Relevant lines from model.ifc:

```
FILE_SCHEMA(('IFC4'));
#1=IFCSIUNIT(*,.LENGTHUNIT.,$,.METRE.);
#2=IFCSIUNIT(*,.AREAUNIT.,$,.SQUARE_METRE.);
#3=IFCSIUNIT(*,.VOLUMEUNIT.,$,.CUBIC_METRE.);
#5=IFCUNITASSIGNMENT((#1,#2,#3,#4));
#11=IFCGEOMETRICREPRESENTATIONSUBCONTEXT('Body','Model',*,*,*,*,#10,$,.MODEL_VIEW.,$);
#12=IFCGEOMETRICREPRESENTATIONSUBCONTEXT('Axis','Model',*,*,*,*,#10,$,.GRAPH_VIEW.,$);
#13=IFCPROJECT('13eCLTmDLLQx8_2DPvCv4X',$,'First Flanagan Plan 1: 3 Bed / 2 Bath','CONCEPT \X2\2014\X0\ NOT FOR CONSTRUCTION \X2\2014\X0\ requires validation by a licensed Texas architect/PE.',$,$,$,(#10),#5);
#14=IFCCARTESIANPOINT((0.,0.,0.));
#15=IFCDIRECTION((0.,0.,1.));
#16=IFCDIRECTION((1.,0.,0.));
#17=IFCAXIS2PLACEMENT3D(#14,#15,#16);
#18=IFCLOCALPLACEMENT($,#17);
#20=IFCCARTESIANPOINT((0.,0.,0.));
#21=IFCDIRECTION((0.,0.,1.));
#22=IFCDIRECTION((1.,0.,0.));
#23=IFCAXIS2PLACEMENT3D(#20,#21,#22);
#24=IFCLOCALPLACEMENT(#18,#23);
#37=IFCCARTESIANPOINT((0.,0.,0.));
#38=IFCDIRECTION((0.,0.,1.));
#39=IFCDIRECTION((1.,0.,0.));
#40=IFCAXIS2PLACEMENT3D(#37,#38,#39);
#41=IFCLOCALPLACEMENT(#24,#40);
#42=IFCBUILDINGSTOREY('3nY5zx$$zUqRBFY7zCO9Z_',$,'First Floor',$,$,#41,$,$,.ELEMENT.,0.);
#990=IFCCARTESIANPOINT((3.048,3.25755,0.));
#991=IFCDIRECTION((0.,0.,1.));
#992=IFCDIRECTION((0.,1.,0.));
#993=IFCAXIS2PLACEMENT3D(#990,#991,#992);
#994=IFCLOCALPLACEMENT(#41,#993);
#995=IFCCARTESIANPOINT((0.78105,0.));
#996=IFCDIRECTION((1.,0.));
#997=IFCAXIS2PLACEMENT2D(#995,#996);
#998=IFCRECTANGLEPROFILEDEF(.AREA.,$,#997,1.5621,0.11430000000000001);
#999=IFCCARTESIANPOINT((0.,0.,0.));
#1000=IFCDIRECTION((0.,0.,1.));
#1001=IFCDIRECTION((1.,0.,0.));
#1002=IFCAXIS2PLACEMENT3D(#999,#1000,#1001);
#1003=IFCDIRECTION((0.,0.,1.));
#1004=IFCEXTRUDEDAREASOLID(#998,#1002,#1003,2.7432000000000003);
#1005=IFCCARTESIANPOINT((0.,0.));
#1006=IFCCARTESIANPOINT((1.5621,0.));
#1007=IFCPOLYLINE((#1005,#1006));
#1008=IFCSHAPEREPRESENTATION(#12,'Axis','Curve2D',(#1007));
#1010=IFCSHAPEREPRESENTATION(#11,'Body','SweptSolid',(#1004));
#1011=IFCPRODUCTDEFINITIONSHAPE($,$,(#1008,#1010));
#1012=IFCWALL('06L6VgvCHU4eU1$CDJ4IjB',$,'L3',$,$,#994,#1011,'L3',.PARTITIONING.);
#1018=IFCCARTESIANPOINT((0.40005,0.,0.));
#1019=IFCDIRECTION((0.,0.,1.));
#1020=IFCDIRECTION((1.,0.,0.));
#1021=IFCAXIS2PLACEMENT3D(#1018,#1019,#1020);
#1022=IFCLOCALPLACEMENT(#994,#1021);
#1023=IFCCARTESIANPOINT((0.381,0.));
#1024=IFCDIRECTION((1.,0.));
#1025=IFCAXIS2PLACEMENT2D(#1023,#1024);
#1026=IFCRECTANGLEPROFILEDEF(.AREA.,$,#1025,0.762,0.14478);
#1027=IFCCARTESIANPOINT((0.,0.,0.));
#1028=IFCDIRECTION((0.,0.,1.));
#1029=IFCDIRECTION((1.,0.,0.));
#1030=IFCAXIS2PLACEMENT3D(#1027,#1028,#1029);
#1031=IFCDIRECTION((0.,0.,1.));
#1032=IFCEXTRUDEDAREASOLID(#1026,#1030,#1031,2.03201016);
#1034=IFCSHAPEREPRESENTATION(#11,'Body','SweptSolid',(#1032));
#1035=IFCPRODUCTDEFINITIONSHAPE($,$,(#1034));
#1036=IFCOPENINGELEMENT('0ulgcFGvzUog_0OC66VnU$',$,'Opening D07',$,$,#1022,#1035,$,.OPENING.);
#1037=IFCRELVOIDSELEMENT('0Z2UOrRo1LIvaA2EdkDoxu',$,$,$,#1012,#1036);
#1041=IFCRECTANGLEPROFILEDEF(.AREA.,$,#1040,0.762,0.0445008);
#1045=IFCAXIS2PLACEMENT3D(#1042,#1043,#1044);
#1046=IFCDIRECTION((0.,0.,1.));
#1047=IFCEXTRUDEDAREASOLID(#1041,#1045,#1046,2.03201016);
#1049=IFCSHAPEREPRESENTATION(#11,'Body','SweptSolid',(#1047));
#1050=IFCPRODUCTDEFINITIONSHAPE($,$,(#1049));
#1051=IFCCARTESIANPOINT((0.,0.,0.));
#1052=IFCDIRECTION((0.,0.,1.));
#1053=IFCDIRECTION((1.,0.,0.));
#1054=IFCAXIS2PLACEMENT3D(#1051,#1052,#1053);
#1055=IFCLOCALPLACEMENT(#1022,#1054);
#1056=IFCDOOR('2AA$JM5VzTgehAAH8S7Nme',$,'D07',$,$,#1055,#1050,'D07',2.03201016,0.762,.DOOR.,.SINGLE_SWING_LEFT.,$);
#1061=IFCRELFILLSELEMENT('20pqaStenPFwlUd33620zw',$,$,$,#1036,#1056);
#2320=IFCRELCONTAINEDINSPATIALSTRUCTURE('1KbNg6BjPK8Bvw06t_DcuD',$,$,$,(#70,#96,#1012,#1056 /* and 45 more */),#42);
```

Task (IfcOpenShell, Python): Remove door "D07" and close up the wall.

```python
import ifcopenshell
import ifcopenshell.api.feature
import ifcopenshell.api.root
import ifcopenshell.geom
import ifcopenshell.util.shape

model = ifcopenshell.open("model.ifc")
settings = ifcopenshell.geom.settings()


def volume(element):
    """Net volume in cubic metres, openings subtracted."""
    shape = ifcopenshell.geom.create_shape(settings, element)
    return ifcopenshell.util.shape.get_volume(shape.geometry)


door = model.by_guid("2AA$JM5VzTgehAAH8S7Nme")
opening = door.FillsVoids[0].RelatingOpeningElement
wall = opening.VoidsElements[0].RelatingBuildingElement
before = volume(wall)

ifcopenshell.api.root.remove_product(model, product=door)
ifcopenshell.api.feature.remove_feature(model, feature=opening)

after = volume(wall)

print(f"wall volume {before:.3f} -> {after:.3f} m3")

model.write("model_v2.ifc")
```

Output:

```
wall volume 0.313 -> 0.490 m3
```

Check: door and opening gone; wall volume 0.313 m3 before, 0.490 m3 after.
